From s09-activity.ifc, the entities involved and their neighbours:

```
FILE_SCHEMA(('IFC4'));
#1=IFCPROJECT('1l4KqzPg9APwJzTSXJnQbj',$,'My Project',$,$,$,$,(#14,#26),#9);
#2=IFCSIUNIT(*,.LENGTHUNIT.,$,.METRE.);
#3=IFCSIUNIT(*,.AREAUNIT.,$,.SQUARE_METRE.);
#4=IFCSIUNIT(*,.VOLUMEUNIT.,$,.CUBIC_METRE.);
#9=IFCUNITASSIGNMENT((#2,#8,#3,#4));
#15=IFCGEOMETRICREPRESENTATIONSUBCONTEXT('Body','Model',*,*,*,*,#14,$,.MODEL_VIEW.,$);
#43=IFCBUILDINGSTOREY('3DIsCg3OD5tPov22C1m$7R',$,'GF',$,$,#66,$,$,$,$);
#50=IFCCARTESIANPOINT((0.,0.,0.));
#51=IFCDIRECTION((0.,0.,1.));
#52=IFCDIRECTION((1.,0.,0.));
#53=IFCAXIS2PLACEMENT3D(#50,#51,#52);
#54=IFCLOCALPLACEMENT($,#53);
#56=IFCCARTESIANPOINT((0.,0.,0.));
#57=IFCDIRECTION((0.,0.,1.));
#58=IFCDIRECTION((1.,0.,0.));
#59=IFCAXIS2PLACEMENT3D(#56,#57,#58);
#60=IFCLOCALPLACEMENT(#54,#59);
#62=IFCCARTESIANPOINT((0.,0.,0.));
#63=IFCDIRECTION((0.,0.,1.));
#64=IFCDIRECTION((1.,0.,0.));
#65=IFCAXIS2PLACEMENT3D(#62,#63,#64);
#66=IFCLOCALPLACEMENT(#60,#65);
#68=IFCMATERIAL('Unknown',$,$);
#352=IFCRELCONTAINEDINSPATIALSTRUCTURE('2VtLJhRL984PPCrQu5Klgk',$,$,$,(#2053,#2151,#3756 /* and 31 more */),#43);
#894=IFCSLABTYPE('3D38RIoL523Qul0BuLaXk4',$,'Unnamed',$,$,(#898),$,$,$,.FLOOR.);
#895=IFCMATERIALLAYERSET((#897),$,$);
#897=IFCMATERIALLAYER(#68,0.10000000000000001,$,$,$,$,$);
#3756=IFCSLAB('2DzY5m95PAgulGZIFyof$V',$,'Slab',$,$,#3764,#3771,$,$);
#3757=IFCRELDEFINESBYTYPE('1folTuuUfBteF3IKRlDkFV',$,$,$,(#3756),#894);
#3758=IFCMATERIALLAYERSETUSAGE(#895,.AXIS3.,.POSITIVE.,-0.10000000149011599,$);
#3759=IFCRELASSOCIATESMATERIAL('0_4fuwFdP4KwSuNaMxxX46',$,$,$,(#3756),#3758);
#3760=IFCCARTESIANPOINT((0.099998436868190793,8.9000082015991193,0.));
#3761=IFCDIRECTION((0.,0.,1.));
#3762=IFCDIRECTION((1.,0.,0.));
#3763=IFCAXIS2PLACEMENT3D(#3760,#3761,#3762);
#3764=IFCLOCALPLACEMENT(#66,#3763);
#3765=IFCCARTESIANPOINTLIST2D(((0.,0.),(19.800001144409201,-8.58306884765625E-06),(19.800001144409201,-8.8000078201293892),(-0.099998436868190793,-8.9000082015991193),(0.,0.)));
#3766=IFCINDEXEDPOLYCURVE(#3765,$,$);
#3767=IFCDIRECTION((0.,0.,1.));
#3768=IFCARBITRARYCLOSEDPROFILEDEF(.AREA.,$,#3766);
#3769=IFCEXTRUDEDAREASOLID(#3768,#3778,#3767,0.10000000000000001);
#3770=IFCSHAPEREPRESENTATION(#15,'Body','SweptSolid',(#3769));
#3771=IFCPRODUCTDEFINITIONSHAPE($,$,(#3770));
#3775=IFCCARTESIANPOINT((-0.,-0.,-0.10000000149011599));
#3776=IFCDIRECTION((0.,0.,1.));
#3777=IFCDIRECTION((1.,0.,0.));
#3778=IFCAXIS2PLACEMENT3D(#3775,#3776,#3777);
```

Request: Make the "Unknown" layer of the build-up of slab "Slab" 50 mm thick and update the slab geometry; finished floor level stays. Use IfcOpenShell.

```python
import ifcopenshell
import ifcopenshell.util.element
import ifcopenshell.util.representation
import ifcopenshell.util.unit

model = ifcopenshell.open("s09-activity.ifc")
unit_scale = ifcopenshell.util.unit.calculate_unit_scale(model)

layer_set = model.by_id(895)
layer = next(l for l in layer_set.MaterialLayers if l.Material and l.Material.Name == "Unknown")
change = 0.05 / unit_scale - layer.LayerThickness
layer.LayerThickness += change

# Geometry does not follow the layer set by itself.
slabs = [e for e in ifcopenshell.util.element.get_elements_by_material(model, layer_set) if e.is_a("IfcSlab")]
for slab in sorted(slabs, key=lambda e: e.id()):
    body = ifcopenshell.util.representation.get_representation(slab, "Model", "Body")
    solid = body.Items[0]
    old_depth = solid.Depth
    solid.Depth += change
    # Extruded upwards: lower the start of the extrusion so the top stays.
    x, y, z = solid.Position.Location.Coordinates
    solid.Position.Location = model.createIfcCartesianPoint((x, y, z - change))
    print(slab.id(), f"{old_depth:g} -> {solid.Depth:g}")

# The layers are counted up from the underside, which has moved.
for usage in {ifcopenshell.util.element.get_material(slab) for slab in slabs}:
    usage.OffsetFromReferenceLine -= change

model.write("s09-activity_v2.ifc")
```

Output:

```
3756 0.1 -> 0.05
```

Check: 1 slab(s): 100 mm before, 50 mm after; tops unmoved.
